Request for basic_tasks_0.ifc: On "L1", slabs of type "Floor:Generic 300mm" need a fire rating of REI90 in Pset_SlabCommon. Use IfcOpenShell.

First a look at what the model holds.

```python
import ifcopenshell
import ifcopenshell.util.element

model = ifcopenshell.open("basic_tasks_0.ifc")
print(model.schema)
storey = next(s for s in model.by_type("IfcBuildingStorey") if s.Name == "L1")
slabs = [e for e in ifcopenshell.util.element.get_decomposition(storey) if e.is_a("IfcSlab")]
seen = {}
for e in slabs:
    element_type = ifcopenshell.util.element.get_type(e)
    key = (element_type.Name if element_type != e and element_type else None, ifcopenshell.util.element.get_pset(e, "Pset_SlabCommon", "FireRating"))
    seen[key] = seen.get(key, 0) + 1
for (name, value), count in sorted(seen.items(), key=str):
    print(count, "x", name, "|", value)
```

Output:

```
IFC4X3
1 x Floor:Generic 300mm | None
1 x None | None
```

```python
import ifcopenshell
import ifcopenshell.api.pset
import ifcopenshell.util.element

model = ifcopenshell.open("basic_tasks_0.ifc")

storey = next(s for s in model.by_type("IfcBuildingStorey") if s.Name == "L1")
slabs = [e for e in ifcopenshell.util.element.get_decomposition(storey) if e.is_a("IfcSlab")]

count = 0
for e in slabs:
    element_type = ifcopenshell.util.element.get_type(e)
    if element_type in (None, e) or element_type.Name != "Floor:Generic 300mm":
        continue
    # add_pset returns the element's existing set when there is one.
    pset = ifcopenshell.api.pset.add_pset(model, product=e, name="Pset_SlabCommon")
    ifcopenshell.api.pset.edit_pset(model, pset=pset, properties={"FireRating": "REI90"})
    count += 1

print(count, "slabs updated")

model.write("basic_tasks_0_updated.ifc")
```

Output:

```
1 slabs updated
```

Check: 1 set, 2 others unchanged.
